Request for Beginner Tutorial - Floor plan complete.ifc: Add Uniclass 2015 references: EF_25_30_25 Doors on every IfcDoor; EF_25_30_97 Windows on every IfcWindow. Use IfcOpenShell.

First a look at what the model holds.

```python
import ifcopenshell

model = ifcopenshell.open("Beginner Tutorial - Floor plan complete.ifc")
print(model.schema)
print("classifications:", [c.Name for c in model.by_type("IfcClassification")])
for ifc_class in ("IfcDoor", "IfcRoof", "IfcStair", "IfcWall", "IfcWindow"):
    print(ifc_class, len(model.by_type(ifc_class)))
```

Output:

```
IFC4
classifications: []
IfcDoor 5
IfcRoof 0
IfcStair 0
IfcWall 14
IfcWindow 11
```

```python
import ifcopenshell
import ifcopenshell.api.classification

model = ifcopenshell.open("Beginner Tutorial - Floor plan complete.ifc")

system = ifcopenshell.api.classification.add_classification(model, classification="Uniclass 2015")

codes = {
    "IfcDoor": ("EF_25_30_25", "Doors"),
    "IfcWindow": ("EF_25_30_97", "Windows"),
}
for ifc_class, (code, name) in codes.items():
    products = model.by_type(ifc_class)
    ifcopenshell.api.classification.add_reference(
        model, products=products, classification=system, identification=code, name=name
    )
    print(code, len(products))

model.write("Beginner Tutorial - Floor plan complete-out.ifc")
```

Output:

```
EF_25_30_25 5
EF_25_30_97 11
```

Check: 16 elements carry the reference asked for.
